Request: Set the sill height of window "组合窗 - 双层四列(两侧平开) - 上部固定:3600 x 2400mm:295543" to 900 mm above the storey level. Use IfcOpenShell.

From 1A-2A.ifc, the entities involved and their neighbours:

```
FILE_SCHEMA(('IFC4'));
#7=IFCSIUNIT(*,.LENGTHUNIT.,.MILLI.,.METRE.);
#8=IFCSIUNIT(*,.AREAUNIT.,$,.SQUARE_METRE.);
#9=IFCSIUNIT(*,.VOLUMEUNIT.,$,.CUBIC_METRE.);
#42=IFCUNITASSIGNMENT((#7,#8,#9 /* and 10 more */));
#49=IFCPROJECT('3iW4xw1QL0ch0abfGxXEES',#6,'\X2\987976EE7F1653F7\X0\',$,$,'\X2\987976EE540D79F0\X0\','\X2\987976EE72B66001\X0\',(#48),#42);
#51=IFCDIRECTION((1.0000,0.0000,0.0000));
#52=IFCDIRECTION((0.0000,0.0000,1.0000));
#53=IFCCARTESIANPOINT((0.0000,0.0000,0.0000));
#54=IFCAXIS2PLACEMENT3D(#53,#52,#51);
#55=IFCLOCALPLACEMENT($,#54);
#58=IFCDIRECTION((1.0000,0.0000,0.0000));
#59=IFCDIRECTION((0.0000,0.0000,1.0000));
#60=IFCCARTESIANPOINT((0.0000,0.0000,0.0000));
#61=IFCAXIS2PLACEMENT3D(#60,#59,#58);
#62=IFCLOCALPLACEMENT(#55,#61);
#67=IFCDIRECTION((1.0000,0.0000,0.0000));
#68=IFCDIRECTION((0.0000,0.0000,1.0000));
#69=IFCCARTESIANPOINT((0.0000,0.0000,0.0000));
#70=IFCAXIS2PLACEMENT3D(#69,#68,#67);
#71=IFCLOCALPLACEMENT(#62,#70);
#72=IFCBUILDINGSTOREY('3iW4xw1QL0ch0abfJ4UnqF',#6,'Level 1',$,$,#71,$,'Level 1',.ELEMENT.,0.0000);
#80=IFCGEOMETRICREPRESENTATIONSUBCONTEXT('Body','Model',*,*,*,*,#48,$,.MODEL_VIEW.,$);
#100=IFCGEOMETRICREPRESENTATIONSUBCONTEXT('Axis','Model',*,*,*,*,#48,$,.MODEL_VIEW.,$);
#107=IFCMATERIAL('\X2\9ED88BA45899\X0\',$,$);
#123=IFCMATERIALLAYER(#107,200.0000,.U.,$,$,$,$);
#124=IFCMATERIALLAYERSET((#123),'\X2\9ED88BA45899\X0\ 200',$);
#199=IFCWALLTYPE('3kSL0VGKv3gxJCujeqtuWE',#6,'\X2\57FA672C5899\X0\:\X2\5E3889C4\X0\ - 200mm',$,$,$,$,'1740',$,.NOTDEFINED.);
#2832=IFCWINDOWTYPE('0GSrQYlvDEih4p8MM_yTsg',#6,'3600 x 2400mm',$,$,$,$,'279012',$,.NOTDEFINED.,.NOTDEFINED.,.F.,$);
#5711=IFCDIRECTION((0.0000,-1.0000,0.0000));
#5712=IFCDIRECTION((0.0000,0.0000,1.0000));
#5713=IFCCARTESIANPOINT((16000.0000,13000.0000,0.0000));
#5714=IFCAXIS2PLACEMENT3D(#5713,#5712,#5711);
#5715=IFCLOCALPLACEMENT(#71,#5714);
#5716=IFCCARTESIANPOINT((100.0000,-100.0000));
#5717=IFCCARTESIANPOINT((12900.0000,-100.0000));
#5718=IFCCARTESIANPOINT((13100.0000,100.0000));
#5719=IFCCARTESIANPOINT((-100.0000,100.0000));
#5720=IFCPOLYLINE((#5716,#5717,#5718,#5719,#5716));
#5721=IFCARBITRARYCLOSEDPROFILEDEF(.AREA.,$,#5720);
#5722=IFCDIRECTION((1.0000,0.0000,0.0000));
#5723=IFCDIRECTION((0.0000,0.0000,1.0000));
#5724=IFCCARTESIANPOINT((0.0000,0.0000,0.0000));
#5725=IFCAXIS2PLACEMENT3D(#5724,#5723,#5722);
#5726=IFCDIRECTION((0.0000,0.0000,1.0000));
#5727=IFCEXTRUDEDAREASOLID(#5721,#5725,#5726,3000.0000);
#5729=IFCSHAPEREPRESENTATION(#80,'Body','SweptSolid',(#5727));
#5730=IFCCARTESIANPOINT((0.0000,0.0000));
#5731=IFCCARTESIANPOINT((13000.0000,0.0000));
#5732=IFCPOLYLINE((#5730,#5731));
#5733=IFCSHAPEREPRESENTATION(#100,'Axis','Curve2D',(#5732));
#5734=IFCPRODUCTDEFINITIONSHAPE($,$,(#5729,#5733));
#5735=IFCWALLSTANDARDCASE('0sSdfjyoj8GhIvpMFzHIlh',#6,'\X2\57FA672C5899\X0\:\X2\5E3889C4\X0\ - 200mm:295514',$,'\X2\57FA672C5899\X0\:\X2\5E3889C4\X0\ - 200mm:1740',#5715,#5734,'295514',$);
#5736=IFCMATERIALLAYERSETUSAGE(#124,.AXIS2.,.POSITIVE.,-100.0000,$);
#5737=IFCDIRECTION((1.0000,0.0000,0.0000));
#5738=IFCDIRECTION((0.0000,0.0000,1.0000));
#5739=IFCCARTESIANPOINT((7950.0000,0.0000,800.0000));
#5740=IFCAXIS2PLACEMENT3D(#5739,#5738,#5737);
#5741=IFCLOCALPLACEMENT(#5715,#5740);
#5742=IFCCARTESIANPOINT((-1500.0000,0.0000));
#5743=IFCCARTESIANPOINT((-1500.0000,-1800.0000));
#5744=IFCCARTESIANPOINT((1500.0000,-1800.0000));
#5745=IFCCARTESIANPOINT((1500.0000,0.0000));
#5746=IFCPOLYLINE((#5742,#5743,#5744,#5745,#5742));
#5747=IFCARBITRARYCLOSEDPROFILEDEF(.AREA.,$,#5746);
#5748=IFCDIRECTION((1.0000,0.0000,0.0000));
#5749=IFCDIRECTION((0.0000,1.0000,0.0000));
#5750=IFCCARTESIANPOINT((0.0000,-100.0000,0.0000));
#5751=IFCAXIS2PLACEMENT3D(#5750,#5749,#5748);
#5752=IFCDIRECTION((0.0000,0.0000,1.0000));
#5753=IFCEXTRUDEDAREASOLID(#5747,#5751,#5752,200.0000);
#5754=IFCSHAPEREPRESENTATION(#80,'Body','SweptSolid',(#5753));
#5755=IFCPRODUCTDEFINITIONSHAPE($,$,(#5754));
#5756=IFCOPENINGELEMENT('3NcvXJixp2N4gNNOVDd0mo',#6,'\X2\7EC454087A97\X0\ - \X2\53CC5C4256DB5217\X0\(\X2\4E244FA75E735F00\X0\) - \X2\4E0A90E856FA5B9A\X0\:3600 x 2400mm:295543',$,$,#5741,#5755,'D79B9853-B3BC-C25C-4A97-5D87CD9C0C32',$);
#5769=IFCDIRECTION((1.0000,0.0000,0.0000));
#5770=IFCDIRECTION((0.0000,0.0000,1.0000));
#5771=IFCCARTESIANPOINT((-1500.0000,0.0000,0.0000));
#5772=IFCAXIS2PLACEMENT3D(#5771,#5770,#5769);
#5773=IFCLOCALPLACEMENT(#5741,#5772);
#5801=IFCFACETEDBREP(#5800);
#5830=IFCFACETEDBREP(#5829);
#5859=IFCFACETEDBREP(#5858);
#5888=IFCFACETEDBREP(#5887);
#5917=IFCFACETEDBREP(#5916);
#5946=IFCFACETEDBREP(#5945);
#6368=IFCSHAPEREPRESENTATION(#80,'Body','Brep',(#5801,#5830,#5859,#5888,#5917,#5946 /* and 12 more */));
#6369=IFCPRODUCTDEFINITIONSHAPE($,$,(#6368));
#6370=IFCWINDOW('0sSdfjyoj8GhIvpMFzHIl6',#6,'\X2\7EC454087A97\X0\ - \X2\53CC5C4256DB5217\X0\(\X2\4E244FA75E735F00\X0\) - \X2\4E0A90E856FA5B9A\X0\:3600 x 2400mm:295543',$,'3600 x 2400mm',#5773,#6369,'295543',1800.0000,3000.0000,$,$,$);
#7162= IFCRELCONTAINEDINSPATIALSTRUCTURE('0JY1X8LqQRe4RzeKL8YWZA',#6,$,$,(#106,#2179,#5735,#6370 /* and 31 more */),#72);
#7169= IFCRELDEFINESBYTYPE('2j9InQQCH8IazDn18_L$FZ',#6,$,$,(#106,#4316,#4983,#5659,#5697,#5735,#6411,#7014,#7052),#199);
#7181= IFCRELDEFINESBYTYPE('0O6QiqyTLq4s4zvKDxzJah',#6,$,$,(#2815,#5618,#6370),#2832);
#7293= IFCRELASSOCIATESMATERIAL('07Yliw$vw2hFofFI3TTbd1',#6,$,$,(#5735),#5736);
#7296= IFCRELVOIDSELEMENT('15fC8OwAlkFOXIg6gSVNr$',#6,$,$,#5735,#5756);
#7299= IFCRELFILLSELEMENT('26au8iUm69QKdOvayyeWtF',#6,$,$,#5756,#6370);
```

```python
import numpy as np
import ifcopenshell
import ifcopenshell.api.geometry
import ifcopenshell.geom
import ifcopenshell.util.element
import ifcopenshell.util.placement
import ifcopenshell.util.shape
import ifcopenshell.util.unit

model = ifcopenshell.open("1A-2A.ifc")
unit_scale = ifcopenshell.util.unit.calculate_unit_scale(model)

window = model.by_guid("0sSdfjyoj8GhIvpMFzHIl6")
opening = window.FillsVoids[0].RelatingOpeningElement
storey = ifcopenshell.util.element.get_container(window, ifc_class="IfcBuildingStorey")
level = ifcopenshell.util.placement.get_local_placement(storey.ObjectPlacement)[2, 3]

# The opening's origin need not be at the sill, so measure its lowest point.
shape = ifcopenshell.geom.create_shape(ifcopenshell.geom.settings(), opening)
bottom = ifcopenshell.util.shape.get_shape_bottom_elevation(shape, shape.geometry) / unit_scale
dz = level + 900.0 - bottom

shift = np.array([0.0, 0.0, dz])
# The window is placed relative to its opening, so it follows when the opening moves.
matrix = ifcopenshell.util.placement.get_local_placement(opening.ObjectPlacement)
matrix[:3, 3] += shift
ifcopenshell.api.geometry.edit_object_placement(
    model, product=opening, matrix=matrix, is_si=False, should_transform_children=True
)

print(f"moved by {dz * unit_scale:+.3f} m")

model.write("1A-2A_updated.ifc")
```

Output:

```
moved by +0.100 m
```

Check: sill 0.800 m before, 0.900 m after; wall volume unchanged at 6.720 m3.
